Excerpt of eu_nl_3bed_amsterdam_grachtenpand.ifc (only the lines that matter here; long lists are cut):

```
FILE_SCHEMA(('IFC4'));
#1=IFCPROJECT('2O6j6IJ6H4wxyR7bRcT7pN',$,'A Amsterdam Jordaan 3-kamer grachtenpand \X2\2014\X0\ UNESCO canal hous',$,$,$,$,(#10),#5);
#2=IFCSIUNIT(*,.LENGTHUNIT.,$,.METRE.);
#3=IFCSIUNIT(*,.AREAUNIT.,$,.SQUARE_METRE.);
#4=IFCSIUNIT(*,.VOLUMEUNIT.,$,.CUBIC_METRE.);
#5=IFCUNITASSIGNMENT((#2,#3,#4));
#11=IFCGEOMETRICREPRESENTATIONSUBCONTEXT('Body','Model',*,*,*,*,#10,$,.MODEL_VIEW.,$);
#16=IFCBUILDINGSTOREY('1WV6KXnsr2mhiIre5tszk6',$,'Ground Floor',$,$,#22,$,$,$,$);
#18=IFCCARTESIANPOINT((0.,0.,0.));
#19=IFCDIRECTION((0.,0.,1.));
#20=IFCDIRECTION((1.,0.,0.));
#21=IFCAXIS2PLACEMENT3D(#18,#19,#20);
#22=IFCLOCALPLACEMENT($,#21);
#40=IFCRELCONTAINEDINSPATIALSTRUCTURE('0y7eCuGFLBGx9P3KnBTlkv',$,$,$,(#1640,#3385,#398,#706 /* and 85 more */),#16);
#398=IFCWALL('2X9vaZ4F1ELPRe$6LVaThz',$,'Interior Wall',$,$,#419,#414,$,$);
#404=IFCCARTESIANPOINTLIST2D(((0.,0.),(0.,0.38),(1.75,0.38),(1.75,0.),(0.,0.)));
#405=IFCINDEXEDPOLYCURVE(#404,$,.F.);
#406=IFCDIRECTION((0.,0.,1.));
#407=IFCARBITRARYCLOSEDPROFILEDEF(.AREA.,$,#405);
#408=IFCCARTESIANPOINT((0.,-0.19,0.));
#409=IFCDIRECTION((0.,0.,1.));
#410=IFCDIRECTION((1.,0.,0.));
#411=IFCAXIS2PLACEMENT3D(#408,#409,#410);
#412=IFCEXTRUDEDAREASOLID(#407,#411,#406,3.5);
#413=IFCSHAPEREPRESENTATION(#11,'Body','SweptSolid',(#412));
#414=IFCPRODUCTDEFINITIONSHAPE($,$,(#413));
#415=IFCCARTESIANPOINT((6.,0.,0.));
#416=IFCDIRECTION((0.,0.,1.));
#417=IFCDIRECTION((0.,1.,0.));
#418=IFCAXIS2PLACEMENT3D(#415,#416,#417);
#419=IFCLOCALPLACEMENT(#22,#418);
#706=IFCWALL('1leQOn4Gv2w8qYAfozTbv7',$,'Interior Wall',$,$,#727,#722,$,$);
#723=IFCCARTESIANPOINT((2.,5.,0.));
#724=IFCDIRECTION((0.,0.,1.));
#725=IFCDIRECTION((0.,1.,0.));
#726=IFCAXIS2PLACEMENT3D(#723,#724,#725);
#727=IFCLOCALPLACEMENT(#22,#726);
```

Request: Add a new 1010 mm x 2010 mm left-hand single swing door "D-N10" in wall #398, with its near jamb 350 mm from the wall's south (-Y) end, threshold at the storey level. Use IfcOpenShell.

```python
import numpy as np
import ifcopenshell
import ifcopenshell.api.feature
import ifcopenshell.api.geometry
import ifcopenshell.api.root
import ifcopenshell.api.spatial
import ifcopenshell.geom
import ifcopenshell.util.element
import ifcopenshell.util.placement
import ifcopenshell.util.representation
import ifcopenshell.util.shape
import ifcopenshell.util.unit

model = ifcopenshell.open("eu_nl_3bed_amsterdam_grachtenpand.ifc")
unit_scale = ifcopenshell.util.unit.calculate_unit_scale(model)
settings = ifcopenshell.geom.settings()


def volume(element):
    """Net volume in cubic metres, openings subtracted."""
    shape = ifcopenshell.geom.create_shape(settings, element)
    return ifcopenshell.util.shape.get_volume(shape.geometry)


wall = model.by_guid("2X9vaZ4F1ELPRe$6LVaThz")
storey = ifcopenshell.util.element.get_container(wall, ifc_class="IfcBuildingStorey")
context = ifcopenshell.util.representation.get_context(model, "Model", "Body", "MODEL_VIEW")
before = volume(wall)

width, height, from_end, sill = 1.01, 2.01, 0.35, 0.0  # metres

# The wall runs along its own X axis, and the end named is its -X end.
wall_shape = ifcopenshell.geom.create_shape(settings, wall)
x, y, z = ifcopenshell.util.shape.get_vertices(wall_shape.geometry).T
start = x.min() + from_end
face, thickness = float(y.min()), float(y.max() - y.min())
wall_matrix = ifcopenshell.util.placement.get_local_placement(wall.ObjectPlacement)
level = ifcopenshell.util.placement.get_local_placement(storey.ObjectPlacement)[2, 3]


def in_wall(x, y):
    """Placement at x, y metres in the wall's axes, at sill height."""
    matrix = wall_matrix.copy()
    matrix[:, 3] = wall_matrix @ np.array([x / unit_scale, y / unit_scale, 0.0, 1.0])
    matrix[2, 3] = level + sill / unit_scale
    return matrix


# Opening: a box that overshoots both wall faces by 50 mm.
opening = ifcopenshell.api.root.create_entity(model, ifc_class="IfcOpeningElement", predefined_type="OPENING")
box = ifcopenshell.api.geometry.add_wall_representation(
    model, context=context, length=width, height=height, thickness=thickness + 0.1
)
ifcopenshell.api.geometry.assign_representation(model, product=opening, representation=box)
ifcopenshell.api.geometry.edit_object_placement(model, product=opening, matrix=in_wall(start, face - 0.05), is_si=False)
ifcopenshell.api.feature.add_feature(model, feature=opening, element=wall)

door = ifcopenshell.api.root.create_entity(model, ifc_class="IfcDoor", name="D-N10", predefined_type="DOOR")
door.OverallWidth, door.OverallHeight = width / unit_scale, height / unit_scale
door.OperationType = "SINGLE_SWING_LEFT"
body = ifcopenshell.api.geometry.add_door_representation(
    model,
    context=context,
    overall_width=door.OverallWidth,
    overall_height=door.OverallHeight,
    operation_type="SINGLE_SWING_LEFT",
    lining_properties={"LiningDepth": thickness / unit_scale, "ThresholdDepth": thickness / unit_scale},
)
ifcopenshell.api.geometry.assign_representation(model, product=door, representation=body)
ifcopenshell.api.spatial.assign_container(model, products=[door], relating_structure=storey)
ifcopenshell.api.feature.add_filling(model, opening=opening, element=door)

# The lining spans the wall, so the door starts at the wall face.
ifcopenshell.api.geometry.edit_object_placement(model, product=door, matrix=in_wall(start, face), is_si=False)

after = volume(wall)

print(f"wall volume {before:.3f} -> {after:.3f} m3")

model.write("eu_nl_3bed_amsterdam_grachtenpand_updated.ifc")
```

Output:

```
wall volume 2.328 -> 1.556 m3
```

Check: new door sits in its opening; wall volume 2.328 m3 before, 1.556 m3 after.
